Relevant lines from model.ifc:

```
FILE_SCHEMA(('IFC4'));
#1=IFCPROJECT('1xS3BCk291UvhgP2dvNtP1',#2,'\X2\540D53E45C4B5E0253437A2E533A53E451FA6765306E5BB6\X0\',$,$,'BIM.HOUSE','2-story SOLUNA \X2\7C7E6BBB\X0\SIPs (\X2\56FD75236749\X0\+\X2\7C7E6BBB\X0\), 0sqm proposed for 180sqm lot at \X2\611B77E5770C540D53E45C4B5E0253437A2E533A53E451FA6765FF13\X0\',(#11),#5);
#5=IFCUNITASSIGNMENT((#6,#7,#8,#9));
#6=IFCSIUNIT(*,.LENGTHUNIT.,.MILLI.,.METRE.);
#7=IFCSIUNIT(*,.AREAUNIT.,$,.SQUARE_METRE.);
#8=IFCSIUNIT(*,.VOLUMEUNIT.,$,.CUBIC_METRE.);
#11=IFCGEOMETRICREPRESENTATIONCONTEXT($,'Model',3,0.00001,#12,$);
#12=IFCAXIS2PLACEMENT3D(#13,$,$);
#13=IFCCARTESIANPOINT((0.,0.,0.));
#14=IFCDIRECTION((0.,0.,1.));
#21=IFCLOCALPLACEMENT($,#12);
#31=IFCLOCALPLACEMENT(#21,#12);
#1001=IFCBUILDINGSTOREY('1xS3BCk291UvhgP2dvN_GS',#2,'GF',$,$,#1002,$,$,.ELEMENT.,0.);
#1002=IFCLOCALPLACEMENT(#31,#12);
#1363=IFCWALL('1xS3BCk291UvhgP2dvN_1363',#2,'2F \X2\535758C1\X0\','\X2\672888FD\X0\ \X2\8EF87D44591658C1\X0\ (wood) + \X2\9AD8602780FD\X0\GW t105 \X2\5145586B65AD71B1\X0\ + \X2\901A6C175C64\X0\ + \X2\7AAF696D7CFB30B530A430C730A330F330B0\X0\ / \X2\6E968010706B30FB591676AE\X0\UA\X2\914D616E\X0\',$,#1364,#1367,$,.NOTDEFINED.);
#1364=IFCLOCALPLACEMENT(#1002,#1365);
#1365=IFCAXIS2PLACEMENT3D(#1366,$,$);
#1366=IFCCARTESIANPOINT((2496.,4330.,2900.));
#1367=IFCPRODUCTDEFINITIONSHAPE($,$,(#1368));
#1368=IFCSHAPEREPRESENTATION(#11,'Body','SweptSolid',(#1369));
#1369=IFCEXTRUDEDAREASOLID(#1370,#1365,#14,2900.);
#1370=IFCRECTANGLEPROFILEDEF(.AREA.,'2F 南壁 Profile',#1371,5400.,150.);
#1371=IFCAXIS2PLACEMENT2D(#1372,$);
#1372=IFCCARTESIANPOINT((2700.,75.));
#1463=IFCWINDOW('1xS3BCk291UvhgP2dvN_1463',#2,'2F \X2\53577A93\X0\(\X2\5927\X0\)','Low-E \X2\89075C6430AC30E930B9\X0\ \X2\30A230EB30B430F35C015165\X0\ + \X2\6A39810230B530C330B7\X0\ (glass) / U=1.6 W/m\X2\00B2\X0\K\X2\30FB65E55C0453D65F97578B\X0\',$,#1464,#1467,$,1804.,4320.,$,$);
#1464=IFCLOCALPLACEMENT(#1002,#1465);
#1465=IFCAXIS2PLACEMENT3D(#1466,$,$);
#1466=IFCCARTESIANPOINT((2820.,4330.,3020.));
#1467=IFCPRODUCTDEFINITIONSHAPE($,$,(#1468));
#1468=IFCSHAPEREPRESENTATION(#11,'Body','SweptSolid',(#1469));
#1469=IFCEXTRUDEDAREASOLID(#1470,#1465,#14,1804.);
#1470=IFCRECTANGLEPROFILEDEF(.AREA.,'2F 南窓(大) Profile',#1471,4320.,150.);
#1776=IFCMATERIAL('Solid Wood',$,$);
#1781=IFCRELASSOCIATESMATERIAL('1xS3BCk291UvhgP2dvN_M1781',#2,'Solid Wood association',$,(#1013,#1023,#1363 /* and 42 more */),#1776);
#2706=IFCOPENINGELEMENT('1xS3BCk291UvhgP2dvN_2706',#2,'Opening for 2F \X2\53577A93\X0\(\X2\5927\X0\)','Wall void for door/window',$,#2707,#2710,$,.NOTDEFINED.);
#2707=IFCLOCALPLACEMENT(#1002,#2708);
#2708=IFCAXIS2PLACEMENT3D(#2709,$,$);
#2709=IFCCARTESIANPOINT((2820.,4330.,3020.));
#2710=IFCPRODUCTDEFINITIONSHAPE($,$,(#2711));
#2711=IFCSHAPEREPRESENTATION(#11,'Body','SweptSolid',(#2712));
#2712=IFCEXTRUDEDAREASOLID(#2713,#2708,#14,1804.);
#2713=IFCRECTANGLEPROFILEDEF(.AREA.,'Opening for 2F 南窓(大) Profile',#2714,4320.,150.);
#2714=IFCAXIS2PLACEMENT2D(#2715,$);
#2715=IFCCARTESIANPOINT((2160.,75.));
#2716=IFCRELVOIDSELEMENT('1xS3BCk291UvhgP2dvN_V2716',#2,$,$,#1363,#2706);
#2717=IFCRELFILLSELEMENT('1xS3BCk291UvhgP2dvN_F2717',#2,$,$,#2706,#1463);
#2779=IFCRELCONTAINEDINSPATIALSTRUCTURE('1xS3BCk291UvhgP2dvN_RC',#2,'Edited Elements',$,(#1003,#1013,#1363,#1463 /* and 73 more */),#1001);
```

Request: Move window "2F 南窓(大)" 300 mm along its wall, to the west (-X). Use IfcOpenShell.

```python
import ifcopenshell
import ifcopenshell.api.geometry
import ifcopenshell.util.placement
import ifcopenshell.util.unit

model = ifcopenshell.open("model.ifc")
unit_scale = ifcopenshell.util.unit.calculate_unit_scale(model)

window = model.by_id(1463)
opening = window.FillsVoids[0].RelatingOpeningElement
wall = opening.VoidsElements[0].RelatingBuildingElement

wall_matrix = ifcopenshell.util.placement.get_local_placement(wall.ObjectPlacement)
shift = wall_matrix[:3, 0] * -0.3 / unit_scale
before = ifcopenshell.util.placement.get_local_placement(window.ObjectPlacement)[:3, 3].copy()

# The window is not placed relative to its opening, so move both.
for product in (opening, window):
    matrix = ifcopenshell.util.placement.get_local_placement(product.ObjectPlacement)
    matrix[:3, 3] += shift
    ifcopenshell.api.geometry.edit_object_placement(model, product=product, matrix=matrix, is_si=False)

after = ifcopenshell.util.placement.get_local_placement(window.ObjectPlacement)[:3, 3]
print("window moved by", (after - before).round(3) + 0.0)

model.write("model-out.ifc")
```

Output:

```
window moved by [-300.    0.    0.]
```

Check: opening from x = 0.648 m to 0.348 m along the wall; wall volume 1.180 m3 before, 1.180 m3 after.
